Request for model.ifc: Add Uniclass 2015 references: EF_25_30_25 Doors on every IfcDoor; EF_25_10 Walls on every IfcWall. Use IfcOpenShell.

First a look at what the model holds.

```python
import ifcopenshell

model = ifcopenshell.open("model.ifc")
print(model.schema)
print("classifications:", [c.Name for c in model.by_type("IfcClassification")])
for ifc_class in ("IfcDoor", "IfcRoof", "IfcStair", "IfcWall", "IfcWindow"):
    print(ifc_class, len(model.by_type(ifc_class)))
```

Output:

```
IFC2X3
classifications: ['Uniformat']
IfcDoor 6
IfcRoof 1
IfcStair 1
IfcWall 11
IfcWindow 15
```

```python
import ifcopenshell
import ifcopenshell.api.classification

model = ifcopenshell.open("model.ifc")

# IFC2X3 requires Source and Edition and has no link from the project to the system.
system = model.create_entity("IfcClassification", Source="NBS", Edition="2015", Name="Uniclass 2015")

codes = {
    "IfcDoor": ("EF_25_30_25", "Doors"),
    "IfcWall": ("EF_25_10", "Walls"),
}
for ifc_class, (code, name) in codes.items():
    products = model.by_type(ifc_class)
    ifcopenshell.api.classification.add_reference(
        model, products=products, classification=system, identification=code, name=name
    )
    print(code, len(products))

model.write("model_v2.ifc")
```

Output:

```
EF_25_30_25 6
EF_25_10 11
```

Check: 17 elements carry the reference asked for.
